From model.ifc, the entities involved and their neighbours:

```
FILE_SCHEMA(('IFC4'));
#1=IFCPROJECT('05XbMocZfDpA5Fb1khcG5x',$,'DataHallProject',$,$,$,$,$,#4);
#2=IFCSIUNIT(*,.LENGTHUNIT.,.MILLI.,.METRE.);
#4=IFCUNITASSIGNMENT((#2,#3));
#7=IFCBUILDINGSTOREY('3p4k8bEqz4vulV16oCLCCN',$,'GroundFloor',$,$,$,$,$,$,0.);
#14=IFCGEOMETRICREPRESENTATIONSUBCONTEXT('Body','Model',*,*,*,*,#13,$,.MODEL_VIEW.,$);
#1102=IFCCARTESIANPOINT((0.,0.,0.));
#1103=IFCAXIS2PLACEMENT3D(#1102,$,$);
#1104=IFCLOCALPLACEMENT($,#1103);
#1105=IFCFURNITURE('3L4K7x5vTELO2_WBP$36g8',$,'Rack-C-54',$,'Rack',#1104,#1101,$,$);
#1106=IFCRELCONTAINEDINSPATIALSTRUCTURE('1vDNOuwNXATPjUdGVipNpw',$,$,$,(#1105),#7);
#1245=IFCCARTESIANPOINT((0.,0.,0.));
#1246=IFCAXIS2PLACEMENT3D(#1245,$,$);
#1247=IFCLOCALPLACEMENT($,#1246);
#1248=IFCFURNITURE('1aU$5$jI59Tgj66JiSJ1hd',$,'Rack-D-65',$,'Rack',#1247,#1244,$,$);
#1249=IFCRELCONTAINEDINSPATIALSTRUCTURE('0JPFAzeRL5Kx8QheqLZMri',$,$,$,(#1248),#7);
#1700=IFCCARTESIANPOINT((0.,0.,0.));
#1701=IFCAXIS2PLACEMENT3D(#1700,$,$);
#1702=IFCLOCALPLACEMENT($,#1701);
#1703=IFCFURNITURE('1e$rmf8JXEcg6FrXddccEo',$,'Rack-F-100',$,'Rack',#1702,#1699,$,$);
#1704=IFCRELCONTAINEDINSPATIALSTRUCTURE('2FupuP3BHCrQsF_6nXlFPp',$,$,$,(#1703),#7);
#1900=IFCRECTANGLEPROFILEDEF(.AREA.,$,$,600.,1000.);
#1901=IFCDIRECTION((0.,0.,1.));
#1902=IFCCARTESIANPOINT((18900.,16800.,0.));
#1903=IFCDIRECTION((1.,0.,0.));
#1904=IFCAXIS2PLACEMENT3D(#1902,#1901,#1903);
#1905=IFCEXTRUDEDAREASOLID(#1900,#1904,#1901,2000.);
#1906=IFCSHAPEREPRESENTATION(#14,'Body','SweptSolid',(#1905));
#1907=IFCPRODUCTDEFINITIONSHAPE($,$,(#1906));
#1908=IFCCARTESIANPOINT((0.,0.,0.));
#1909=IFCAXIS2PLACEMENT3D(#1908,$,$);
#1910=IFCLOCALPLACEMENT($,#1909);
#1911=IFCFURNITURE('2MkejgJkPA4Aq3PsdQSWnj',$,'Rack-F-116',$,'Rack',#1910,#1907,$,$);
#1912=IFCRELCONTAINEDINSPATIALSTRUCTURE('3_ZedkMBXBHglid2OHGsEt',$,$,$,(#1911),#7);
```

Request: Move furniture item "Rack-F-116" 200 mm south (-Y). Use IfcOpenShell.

```python
import ifcopenshell
import ifcopenshell.api.geometry
import ifcopenshell.util.placement

model = ifcopenshell.open("model.ifc")

item = model.by_guid("2MkejgJkPA4Aq3PsdQSWnj")
matrix = ifcopenshell.util.placement.get_local_placement(item.ObjectPlacement)
matrix[1, 3] -= 200.0
ifcopenshell.api.geometry.edit_object_placement(model, product=item, matrix=matrix, is_si=False)

print(ifcopenshell.util.placement.get_local_placement(item.ObjectPlacement).round(3) + 0.0)

model.write("model-out.ifc")
```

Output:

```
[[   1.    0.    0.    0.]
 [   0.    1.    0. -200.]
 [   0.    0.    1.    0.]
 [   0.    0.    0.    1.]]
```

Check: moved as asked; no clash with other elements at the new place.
